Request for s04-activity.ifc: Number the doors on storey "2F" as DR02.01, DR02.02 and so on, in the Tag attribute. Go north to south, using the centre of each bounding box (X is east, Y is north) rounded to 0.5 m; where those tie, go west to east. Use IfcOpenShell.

First a look at what the model holds.

```python
import ifcopenshell
import ifcopenshell.util.element
import ifcopenshell.util.placement

model = ifcopenshell.open("s04-activity.ifc")
print(model.schema)
storey = next(s for s in model.by_type("IfcBuildingStorey") if s.Name == "2F")
doors = [e for e in ifcopenshell.util.element.get_decomposition(storey) if e.is_a("IfcDoor")]
for e in sorted(doors, key=lambda e: e.id()):
    origin = ifcopenshell.util.placement.get_local_placement(e.ObjectPlacement)[:3, 3]
    print(e.id(), e.Tag, e.Name, origin.round(2) + 0.0, sep=" | ")
```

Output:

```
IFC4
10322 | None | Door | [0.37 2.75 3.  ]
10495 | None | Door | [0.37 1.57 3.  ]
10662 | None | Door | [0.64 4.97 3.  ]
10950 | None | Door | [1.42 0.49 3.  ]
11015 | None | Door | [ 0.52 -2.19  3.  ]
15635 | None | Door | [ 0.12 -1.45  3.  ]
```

```python
import ifcopenshell
import ifcopenshell.geom
import ifcopenshell.util.element
import ifcopenshell.util.shape

model = ifcopenshell.open("s04-activity.ifc")
settings = ifcopenshell.geom.settings()
settings.set("use-world-coords", True)


def centre(element):
    shape = ifcopenshell.geom.create_shape(settings, element)
    return ifcopenshell.util.shape.get_bbox_centroid(shape.geometry)


storey = next(s for s in model.by_type("IfcBuildingStorey") if s.Name == "2F")
doors = [e for e in ifcopenshell.util.element.get_decomposition(storey) if e.is_a("IfcDoor")]

# Insertion points can sit at a corner or the storey origin, so sort by the geometry (in metres).
centres = {e: centre(e) for e in doors}
doors.sort(key=lambda e: (-round(centres[e][1] / 0.5), centres[e][0]))

for i, e in enumerate(doors, start=1):
    number = f"DR02.{i:02d}"
    e.Tag = number
    print(e.id(), number)

model.write("s04-activity_v2.ifc")
```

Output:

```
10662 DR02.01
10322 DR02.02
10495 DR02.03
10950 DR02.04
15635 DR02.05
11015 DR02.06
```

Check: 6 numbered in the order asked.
